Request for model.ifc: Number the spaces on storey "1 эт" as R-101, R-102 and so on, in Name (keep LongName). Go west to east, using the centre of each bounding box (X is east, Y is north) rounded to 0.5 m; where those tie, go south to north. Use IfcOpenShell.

First a look at what the model holds.

```python
import ifcopenshell
import ifcopenshell.util.element
import ifcopenshell.util.placement

model = ifcopenshell.open("model.ifc")
print(model.schema)
storey = next(s for s in model.by_type("IfcBuildingStorey") if s.Name == "1 эт")
spaces = [e for e in ifcopenshell.util.element.get_decomposition(storey) if e.is_a("IfcSpace")]
for e in sorted(spaces, key=lambda e: e.id()):
    origin = ifcopenshell.util.placement.get_local_placement(e.ObjectPlacement)[:3, 3]
    print(e.id(), e.Name, e.LongName, origin.round(2) + 0.0, sep=" | ")
```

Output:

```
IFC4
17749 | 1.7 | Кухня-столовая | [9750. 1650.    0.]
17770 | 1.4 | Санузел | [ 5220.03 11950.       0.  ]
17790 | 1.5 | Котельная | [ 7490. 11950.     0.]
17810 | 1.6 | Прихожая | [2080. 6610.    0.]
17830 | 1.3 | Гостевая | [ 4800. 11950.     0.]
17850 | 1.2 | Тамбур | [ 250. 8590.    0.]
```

```python
import ifcopenshell
import ifcopenshell.geom
import ifcopenshell.util.element
import ifcopenshell.util.shape

model = ifcopenshell.open("model.ifc")
settings = ifcopenshell.geom.settings()
settings.set("use-world-coords", True)


def centre(element):
    shape = ifcopenshell.geom.create_shape(settings, element)
    return ifcopenshell.util.shape.get_bbox_centroid(shape.geometry)


storey = next(s for s in model.by_type("IfcBuildingStorey") if s.Name == "1 эт")
spaces = [e for e in ifcopenshell.util.element.get_decomposition(storey) if e.is_a("IfcSpace")]

# Insertion points can sit at a corner or the storey origin, so sort by the geometry (in metres).
centres = {e: centre(e) for e in spaces}
spaces.sort(key=lambda e: (round(centres[e][0] / 0.5), centres[e][1]))

for i, e in enumerate(spaces, start=1):
    number = f"R-1{i:02d}"
    e.Name = number
    print(e.id(), number)

model.write("model_v2.ifc")
```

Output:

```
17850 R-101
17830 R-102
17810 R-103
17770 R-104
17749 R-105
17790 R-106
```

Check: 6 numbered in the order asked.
